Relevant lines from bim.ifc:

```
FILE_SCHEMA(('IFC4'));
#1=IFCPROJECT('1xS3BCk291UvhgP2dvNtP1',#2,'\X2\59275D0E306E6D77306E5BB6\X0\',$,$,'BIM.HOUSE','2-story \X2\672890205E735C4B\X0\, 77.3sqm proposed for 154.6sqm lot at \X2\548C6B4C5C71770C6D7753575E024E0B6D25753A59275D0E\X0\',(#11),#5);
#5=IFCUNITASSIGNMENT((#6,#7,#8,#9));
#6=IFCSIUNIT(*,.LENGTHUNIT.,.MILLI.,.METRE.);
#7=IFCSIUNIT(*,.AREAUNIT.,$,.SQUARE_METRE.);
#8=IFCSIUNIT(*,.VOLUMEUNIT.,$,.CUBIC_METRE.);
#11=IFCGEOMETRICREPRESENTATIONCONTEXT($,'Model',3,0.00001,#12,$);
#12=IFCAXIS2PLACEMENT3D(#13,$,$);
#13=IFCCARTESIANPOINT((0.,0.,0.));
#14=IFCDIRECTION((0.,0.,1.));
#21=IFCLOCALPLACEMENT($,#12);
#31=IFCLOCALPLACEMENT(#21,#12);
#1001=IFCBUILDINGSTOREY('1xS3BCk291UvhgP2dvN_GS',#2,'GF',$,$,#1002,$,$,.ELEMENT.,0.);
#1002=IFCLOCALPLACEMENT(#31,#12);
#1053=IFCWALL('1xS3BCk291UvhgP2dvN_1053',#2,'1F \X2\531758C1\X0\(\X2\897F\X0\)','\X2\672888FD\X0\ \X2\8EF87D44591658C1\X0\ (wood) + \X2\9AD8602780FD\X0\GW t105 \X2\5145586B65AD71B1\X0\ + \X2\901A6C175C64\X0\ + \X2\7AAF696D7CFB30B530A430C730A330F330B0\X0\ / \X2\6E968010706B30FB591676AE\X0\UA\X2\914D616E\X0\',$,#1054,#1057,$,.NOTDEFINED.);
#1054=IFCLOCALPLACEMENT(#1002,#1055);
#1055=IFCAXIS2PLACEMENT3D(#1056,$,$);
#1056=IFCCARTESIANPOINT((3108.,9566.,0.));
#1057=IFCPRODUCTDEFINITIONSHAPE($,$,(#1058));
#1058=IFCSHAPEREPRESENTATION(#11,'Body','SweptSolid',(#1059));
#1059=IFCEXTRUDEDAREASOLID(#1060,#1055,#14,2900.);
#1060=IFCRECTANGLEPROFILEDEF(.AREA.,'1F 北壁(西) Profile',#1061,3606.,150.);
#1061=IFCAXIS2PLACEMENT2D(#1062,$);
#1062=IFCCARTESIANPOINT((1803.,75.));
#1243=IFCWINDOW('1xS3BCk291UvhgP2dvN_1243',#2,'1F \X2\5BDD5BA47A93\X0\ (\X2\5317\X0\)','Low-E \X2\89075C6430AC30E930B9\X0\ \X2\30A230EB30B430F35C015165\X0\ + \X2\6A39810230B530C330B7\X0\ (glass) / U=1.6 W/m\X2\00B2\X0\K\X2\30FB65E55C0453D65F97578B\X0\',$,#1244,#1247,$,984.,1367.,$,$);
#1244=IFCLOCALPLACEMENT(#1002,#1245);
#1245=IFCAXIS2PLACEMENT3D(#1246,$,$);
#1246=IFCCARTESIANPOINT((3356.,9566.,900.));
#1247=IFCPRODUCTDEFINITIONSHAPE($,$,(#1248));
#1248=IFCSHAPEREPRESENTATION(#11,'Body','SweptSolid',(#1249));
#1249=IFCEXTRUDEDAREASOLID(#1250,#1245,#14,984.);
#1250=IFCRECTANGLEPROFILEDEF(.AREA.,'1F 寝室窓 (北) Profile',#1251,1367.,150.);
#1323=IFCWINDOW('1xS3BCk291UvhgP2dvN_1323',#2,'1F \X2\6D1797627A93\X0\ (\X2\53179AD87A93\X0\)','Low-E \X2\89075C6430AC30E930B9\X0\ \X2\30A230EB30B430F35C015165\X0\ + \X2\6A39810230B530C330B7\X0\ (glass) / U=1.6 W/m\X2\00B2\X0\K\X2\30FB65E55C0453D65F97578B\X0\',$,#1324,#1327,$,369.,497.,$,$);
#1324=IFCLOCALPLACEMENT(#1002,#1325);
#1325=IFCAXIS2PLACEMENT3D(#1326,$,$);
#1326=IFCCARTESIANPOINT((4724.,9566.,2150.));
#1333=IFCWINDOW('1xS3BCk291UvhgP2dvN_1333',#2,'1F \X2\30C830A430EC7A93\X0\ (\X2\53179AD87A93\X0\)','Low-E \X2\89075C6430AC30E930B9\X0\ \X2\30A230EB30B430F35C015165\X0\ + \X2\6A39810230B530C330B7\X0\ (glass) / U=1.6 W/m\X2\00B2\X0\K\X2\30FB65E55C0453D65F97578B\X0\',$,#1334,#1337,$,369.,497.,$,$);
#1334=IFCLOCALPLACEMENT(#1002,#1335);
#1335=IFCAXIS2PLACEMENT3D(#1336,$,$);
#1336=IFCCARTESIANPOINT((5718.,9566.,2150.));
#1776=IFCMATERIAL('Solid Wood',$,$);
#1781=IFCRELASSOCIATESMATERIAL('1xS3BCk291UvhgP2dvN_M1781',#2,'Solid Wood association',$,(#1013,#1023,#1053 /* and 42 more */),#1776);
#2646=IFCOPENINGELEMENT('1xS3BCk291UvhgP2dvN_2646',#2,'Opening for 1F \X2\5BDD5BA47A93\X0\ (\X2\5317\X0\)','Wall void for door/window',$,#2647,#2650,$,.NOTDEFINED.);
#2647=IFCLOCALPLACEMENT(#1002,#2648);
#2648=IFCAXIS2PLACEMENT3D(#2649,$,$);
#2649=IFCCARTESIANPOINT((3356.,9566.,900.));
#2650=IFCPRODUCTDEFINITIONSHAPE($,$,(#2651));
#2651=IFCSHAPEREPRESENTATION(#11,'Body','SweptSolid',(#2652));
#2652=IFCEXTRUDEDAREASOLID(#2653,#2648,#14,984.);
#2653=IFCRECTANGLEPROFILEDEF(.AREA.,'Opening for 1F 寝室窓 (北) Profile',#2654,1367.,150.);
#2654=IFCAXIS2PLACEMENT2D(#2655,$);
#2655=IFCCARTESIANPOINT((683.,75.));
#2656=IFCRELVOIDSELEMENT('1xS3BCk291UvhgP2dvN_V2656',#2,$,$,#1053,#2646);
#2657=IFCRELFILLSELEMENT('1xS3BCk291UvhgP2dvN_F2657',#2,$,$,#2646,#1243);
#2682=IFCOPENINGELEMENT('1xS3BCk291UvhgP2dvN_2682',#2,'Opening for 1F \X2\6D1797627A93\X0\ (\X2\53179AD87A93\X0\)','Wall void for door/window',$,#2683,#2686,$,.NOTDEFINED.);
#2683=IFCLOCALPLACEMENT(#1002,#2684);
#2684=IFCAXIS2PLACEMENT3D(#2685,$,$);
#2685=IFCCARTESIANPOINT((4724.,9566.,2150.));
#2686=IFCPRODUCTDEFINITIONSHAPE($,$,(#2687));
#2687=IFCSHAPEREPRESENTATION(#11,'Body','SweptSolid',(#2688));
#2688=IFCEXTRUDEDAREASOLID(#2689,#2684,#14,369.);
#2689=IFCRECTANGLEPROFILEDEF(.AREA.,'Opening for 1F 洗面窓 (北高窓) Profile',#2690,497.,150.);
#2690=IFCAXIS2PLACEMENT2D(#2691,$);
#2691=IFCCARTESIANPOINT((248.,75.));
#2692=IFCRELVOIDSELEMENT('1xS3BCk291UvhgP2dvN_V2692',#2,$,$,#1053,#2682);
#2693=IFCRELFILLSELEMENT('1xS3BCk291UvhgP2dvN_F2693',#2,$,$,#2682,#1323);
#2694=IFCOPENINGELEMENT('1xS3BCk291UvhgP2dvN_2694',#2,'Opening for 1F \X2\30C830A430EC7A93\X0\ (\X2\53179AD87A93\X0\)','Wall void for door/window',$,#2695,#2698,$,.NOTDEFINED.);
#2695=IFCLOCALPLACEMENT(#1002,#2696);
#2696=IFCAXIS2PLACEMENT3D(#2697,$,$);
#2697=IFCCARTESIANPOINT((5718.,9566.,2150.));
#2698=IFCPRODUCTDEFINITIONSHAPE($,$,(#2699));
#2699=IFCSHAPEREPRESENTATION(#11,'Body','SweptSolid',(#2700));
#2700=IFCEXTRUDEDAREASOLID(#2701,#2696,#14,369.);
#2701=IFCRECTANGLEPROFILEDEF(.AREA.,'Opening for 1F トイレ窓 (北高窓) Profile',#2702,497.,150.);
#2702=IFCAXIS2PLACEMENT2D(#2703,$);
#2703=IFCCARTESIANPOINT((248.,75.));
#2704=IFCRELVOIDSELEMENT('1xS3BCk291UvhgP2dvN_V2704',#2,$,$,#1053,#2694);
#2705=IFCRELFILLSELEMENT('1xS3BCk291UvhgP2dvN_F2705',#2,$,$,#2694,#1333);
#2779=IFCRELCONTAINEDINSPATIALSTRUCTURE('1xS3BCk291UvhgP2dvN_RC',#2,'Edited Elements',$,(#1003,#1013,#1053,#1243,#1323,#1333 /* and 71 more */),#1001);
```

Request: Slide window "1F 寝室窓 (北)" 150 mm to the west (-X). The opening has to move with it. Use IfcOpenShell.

```python
import ifcopenshell
import ifcopenshell.api.geometry
import ifcopenshell.util.placement
import ifcopenshell.util.unit

model = ifcopenshell.open("bim.ifc")
unit_scale = ifcopenshell.util.unit.calculate_unit_scale(model)

window = model.by_id(1243)
opening = window.FillsVoids[0].RelatingOpeningElement
wall = opening.VoidsElements[0].RelatingBuildingElement

wall_matrix = ifcopenshell.util.placement.get_local_placement(wall.ObjectPlacement)
shift = wall_matrix[:3, 0] * -0.15 / unit_scale
before = ifcopenshell.util.placement.get_local_placement(window.ObjectPlacement)[:3, 3].copy()

# The window is not placed relative to its opening, so move both.
for product in (opening, window):
    matrix = ifcopenshell.util.placement.get_local_placement(product.ObjectPlacement)
    matrix[:3, 3] += shift
    ifcopenshell.api.geometry.edit_object_placement(model, product=product, matrix=matrix, is_si=False)

after = ifcopenshell.util.placement.get_local_placement(window.ObjectPlacement)[:3, 3]
print("window moved by", (after - before).round(3) + 0.0)

model.write("bim_edited.ifc")
```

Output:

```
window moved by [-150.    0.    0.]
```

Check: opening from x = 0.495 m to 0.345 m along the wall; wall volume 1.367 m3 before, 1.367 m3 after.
